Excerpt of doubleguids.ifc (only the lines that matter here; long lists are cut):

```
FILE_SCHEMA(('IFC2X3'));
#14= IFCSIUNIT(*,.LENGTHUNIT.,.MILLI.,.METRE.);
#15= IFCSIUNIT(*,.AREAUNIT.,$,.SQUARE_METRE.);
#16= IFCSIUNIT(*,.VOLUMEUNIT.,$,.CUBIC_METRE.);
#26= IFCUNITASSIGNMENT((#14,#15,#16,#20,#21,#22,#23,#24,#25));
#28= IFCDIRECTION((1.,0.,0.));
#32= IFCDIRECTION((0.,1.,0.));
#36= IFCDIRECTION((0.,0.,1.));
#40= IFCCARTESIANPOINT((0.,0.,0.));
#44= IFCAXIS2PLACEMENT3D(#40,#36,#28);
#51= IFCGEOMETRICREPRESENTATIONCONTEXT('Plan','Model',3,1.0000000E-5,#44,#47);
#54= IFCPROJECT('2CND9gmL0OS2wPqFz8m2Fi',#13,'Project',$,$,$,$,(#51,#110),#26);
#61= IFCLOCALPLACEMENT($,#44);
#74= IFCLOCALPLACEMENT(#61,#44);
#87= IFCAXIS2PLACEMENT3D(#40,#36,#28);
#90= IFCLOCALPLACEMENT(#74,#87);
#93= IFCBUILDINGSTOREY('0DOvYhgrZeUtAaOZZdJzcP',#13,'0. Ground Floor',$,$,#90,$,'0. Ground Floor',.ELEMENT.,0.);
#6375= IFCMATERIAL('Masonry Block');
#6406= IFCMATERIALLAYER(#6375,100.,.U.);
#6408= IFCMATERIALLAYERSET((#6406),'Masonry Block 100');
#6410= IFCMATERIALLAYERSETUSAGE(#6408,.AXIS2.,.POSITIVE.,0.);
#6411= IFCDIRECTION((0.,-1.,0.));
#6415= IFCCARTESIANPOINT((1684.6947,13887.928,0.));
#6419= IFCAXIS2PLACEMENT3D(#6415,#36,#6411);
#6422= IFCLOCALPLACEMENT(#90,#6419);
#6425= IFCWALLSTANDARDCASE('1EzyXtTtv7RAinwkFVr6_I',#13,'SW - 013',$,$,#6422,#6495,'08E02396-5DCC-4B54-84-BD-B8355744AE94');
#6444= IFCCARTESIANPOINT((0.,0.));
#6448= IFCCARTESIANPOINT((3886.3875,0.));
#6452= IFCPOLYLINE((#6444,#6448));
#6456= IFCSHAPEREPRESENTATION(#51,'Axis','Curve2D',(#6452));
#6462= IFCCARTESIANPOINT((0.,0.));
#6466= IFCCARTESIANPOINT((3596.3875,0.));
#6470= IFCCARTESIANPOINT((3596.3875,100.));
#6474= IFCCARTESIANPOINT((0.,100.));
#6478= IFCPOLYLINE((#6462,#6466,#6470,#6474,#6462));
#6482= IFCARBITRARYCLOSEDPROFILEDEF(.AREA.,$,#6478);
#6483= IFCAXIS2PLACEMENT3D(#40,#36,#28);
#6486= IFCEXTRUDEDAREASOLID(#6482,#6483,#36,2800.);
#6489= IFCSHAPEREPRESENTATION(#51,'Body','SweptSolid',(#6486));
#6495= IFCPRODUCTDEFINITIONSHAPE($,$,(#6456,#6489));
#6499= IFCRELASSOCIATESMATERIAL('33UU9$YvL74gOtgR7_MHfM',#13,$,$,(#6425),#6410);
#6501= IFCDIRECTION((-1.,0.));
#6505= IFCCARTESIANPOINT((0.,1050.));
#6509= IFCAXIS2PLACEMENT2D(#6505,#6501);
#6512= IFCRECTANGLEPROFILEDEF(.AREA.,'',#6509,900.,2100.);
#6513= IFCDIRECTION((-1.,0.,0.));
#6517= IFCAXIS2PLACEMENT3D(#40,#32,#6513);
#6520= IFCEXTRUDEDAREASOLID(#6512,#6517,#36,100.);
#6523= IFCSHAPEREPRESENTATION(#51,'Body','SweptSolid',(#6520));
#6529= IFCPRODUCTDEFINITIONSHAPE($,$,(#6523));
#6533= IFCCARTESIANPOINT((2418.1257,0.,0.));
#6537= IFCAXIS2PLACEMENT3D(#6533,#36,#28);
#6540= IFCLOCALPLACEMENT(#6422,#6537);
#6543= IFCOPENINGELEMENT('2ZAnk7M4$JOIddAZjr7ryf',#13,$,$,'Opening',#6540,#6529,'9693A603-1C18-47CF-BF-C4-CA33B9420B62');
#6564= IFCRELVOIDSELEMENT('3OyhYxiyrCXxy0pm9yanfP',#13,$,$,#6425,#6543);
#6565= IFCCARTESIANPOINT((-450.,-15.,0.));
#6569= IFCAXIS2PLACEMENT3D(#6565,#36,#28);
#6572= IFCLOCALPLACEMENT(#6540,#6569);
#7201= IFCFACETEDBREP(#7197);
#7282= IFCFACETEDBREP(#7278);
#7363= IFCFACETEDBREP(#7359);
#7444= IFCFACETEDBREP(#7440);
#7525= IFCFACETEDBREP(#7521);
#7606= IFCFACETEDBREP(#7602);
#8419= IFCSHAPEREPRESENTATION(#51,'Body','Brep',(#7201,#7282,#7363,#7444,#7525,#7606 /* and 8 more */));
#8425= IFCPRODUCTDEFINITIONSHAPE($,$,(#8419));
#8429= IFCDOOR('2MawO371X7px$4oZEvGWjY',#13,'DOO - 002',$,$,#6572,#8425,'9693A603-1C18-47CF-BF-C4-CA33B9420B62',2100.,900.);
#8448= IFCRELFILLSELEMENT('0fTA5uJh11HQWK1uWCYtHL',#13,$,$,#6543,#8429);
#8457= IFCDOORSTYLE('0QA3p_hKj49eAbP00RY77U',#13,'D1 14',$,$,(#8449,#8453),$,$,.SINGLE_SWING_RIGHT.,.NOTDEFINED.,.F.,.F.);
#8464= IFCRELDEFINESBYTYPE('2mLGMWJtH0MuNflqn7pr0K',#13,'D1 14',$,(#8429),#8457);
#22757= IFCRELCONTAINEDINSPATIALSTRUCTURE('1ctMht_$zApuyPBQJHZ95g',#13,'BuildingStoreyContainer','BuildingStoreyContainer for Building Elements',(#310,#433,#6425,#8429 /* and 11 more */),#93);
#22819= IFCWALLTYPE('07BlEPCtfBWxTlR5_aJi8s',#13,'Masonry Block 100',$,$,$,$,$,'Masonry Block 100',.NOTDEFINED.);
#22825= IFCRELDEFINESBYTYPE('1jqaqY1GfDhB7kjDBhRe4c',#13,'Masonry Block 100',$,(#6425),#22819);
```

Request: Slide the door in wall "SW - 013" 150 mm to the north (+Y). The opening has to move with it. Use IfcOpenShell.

```python
import ifcopenshell
import ifcopenshell.api.geometry
import ifcopenshell.util.placement
import ifcopenshell.util.unit

model = ifcopenshell.open("doubleguids.ifc")
unit_scale = ifcopenshell.util.unit.calculate_unit_scale(model)

door = model.by_guid("2MawO371X7px$4oZEvGWjY")
opening = door.FillsVoids[0].RelatingOpeningElement
wall = opening.VoidsElements[0].RelatingBuildingElement

wall_matrix = ifcopenshell.util.placement.get_local_placement(wall.ObjectPlacement)
shift = wall_matrix[:3, 0] * -0.15 / unit_scale
before = ifcopenshell.util.placement.get_local_placement(door.ObjectPlacement)[:3, 3].copy()

# The door is placed relative to its opening, so it follows when the opening moves.
matrix = ifcopenshell.util.placement.get_local_placement(opening.ObjectPlacement)
matrix[:3, 3] += shift
ifcopenshell.api.geometry.edit_object_placement(
    model, product=opening, matrix=matrix, is_si=False, should_transform_children=True
)

after = ifcopenshell.util.placement.get_local_placement(door.ObjectPlacement)[:3, 3]
print("door moved by", (after - before).round(3) + 0.0)

model.write("doubleguids-out.ifc")
```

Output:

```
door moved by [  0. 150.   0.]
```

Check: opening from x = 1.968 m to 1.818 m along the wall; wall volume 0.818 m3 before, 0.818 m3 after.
